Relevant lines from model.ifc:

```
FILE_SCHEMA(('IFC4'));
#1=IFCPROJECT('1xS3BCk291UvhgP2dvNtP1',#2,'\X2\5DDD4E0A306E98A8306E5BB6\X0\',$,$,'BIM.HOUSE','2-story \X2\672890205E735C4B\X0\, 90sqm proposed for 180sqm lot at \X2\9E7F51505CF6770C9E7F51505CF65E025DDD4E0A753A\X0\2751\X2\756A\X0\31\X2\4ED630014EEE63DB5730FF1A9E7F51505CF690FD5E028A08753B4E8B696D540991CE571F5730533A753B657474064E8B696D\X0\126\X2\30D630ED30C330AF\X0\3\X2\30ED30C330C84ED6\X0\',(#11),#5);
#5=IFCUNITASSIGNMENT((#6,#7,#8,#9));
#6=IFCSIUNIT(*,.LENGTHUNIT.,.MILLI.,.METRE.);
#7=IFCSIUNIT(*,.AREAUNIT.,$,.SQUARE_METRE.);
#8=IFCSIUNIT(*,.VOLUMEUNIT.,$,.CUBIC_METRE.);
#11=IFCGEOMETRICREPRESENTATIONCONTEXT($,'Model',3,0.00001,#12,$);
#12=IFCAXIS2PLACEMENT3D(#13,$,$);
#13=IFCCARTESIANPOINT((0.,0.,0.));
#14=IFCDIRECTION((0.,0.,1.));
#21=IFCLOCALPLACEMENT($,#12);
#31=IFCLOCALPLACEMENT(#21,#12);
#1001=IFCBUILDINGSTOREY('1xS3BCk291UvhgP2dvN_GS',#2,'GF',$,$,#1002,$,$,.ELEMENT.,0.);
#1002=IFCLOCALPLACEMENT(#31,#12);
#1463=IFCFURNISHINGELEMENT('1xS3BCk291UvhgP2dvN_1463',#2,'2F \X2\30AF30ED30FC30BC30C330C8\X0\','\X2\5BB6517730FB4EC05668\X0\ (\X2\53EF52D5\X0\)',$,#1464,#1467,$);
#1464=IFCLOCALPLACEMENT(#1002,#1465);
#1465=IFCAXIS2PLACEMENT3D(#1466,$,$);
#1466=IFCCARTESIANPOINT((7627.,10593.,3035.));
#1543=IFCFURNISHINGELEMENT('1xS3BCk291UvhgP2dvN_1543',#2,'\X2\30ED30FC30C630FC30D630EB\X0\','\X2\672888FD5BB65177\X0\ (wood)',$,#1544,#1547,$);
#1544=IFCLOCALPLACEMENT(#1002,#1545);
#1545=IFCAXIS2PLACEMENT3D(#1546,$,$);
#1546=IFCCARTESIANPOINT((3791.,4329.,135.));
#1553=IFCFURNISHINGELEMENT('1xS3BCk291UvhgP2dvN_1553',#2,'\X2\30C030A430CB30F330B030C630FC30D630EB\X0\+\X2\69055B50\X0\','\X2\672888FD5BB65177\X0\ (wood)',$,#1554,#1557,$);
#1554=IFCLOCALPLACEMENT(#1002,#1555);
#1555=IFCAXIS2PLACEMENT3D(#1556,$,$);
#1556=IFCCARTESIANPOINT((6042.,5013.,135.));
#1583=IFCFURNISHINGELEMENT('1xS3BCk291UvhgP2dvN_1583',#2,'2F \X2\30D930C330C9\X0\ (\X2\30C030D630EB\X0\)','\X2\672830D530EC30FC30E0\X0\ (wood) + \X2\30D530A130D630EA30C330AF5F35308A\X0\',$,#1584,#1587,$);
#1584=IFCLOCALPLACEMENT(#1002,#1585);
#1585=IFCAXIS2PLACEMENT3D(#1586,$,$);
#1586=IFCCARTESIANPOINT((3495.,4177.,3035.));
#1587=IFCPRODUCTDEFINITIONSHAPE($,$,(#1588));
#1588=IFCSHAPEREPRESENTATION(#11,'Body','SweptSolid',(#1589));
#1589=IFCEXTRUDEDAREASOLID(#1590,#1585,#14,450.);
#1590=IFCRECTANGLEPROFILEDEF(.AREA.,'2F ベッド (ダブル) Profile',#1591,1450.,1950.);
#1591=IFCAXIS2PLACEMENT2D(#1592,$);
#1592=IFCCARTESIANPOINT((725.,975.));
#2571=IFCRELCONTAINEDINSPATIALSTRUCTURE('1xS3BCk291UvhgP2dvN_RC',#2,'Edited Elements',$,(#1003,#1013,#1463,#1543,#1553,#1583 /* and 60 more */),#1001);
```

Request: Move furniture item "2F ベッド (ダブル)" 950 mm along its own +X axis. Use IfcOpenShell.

```python
import ifcopenshell
import ifcopenshell.api.geometry
import ifcopenshell.util.placement

model = ifcopenshell.open("model.ifc")

item = model.by_guid("1xS3BCk291UvhgP2dvN_1583")
matrix = ifcopenshell.util.placement.get_local_placement(item.ObjectPlacement)
matrix[:3, 3] += matrix[:3, 0] * 950.0
ifcopenshell.api.geometry.edit_object_placement(model, product=item, matrix=matrix, is_si=False)

print(ifcopenshell.util.placement.get_local_placement(item.ObjectPlacement).round(3) + 0.0)

model.write("model_rev.ifc")
```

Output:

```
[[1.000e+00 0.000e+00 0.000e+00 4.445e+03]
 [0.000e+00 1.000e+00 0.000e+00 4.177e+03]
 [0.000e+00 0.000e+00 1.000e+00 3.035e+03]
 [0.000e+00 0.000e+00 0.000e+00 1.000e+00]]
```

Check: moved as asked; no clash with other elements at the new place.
